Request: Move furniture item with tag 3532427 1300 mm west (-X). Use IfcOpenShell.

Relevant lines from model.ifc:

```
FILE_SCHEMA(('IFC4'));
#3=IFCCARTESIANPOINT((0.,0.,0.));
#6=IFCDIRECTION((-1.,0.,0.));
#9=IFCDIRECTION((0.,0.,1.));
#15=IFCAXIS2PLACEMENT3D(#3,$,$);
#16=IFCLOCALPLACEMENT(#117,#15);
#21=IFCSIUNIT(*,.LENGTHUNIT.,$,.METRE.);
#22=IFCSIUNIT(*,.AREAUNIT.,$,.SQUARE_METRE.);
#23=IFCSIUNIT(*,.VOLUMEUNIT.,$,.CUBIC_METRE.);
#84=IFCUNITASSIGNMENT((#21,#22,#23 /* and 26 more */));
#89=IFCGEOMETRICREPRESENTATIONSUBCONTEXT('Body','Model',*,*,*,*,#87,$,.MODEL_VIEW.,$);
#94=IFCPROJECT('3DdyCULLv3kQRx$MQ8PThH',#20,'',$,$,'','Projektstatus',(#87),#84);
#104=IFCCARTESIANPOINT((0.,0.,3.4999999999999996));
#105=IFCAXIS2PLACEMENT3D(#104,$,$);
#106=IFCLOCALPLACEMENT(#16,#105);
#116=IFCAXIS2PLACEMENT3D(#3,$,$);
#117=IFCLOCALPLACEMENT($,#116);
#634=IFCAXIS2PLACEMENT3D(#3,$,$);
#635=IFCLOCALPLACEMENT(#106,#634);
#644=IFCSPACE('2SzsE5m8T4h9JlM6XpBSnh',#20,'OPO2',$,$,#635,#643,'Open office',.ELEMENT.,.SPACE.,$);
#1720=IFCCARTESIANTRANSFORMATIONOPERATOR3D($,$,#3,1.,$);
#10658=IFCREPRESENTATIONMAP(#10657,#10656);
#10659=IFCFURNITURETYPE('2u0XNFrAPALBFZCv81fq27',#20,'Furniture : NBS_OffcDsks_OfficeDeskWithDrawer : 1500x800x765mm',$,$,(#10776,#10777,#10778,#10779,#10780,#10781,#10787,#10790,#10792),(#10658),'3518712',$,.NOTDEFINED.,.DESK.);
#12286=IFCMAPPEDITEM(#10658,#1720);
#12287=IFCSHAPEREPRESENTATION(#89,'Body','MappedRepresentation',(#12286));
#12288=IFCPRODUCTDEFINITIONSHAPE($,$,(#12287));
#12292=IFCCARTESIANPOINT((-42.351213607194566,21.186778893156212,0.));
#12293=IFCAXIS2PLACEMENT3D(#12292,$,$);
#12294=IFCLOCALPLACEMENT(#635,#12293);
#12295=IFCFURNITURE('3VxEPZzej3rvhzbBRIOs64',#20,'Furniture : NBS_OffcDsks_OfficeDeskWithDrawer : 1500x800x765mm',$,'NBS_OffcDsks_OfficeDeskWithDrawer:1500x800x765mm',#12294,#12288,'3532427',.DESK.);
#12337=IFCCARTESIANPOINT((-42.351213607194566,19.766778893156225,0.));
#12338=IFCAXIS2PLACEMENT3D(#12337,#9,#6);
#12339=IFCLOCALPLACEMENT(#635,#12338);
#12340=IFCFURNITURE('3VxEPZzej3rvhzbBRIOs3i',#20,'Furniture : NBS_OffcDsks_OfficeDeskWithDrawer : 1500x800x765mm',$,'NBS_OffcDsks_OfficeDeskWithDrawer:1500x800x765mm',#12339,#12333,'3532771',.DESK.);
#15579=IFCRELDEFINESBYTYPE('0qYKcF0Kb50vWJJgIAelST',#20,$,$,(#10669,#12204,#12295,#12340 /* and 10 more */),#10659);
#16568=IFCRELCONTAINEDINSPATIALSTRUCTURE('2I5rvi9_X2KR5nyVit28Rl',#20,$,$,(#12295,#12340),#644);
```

```python
import ifcopenshell
import ifcopenshell.api.geometry
import ifcopenshell.util.placement
import ifcopenshell.util.unit

model = ifcopenshell.open("model.ifc")
unit_scale = ifcopenshell.util.unit.calculate_unit_scale(model)

item = model.by_guid("3VxEPZzej3rvhzbBRIOs64")
matrix = ifcopenshell.util.placement.get_local_placement(item.ObjectPlacement)
matrix[0, 3] -= 1.3 / unit_scale
ifcopenshell.api.geometry.edit_object_placement(model, product=item, matrix=matrix, is_si=False)

print(ifcopenshell.util.placement.get_local_placement(item.ObjectPlacement).round(3) + 0.0)

model.write("model_rev.ifc")
```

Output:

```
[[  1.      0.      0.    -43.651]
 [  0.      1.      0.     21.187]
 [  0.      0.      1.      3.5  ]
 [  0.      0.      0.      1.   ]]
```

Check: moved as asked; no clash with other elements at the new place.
